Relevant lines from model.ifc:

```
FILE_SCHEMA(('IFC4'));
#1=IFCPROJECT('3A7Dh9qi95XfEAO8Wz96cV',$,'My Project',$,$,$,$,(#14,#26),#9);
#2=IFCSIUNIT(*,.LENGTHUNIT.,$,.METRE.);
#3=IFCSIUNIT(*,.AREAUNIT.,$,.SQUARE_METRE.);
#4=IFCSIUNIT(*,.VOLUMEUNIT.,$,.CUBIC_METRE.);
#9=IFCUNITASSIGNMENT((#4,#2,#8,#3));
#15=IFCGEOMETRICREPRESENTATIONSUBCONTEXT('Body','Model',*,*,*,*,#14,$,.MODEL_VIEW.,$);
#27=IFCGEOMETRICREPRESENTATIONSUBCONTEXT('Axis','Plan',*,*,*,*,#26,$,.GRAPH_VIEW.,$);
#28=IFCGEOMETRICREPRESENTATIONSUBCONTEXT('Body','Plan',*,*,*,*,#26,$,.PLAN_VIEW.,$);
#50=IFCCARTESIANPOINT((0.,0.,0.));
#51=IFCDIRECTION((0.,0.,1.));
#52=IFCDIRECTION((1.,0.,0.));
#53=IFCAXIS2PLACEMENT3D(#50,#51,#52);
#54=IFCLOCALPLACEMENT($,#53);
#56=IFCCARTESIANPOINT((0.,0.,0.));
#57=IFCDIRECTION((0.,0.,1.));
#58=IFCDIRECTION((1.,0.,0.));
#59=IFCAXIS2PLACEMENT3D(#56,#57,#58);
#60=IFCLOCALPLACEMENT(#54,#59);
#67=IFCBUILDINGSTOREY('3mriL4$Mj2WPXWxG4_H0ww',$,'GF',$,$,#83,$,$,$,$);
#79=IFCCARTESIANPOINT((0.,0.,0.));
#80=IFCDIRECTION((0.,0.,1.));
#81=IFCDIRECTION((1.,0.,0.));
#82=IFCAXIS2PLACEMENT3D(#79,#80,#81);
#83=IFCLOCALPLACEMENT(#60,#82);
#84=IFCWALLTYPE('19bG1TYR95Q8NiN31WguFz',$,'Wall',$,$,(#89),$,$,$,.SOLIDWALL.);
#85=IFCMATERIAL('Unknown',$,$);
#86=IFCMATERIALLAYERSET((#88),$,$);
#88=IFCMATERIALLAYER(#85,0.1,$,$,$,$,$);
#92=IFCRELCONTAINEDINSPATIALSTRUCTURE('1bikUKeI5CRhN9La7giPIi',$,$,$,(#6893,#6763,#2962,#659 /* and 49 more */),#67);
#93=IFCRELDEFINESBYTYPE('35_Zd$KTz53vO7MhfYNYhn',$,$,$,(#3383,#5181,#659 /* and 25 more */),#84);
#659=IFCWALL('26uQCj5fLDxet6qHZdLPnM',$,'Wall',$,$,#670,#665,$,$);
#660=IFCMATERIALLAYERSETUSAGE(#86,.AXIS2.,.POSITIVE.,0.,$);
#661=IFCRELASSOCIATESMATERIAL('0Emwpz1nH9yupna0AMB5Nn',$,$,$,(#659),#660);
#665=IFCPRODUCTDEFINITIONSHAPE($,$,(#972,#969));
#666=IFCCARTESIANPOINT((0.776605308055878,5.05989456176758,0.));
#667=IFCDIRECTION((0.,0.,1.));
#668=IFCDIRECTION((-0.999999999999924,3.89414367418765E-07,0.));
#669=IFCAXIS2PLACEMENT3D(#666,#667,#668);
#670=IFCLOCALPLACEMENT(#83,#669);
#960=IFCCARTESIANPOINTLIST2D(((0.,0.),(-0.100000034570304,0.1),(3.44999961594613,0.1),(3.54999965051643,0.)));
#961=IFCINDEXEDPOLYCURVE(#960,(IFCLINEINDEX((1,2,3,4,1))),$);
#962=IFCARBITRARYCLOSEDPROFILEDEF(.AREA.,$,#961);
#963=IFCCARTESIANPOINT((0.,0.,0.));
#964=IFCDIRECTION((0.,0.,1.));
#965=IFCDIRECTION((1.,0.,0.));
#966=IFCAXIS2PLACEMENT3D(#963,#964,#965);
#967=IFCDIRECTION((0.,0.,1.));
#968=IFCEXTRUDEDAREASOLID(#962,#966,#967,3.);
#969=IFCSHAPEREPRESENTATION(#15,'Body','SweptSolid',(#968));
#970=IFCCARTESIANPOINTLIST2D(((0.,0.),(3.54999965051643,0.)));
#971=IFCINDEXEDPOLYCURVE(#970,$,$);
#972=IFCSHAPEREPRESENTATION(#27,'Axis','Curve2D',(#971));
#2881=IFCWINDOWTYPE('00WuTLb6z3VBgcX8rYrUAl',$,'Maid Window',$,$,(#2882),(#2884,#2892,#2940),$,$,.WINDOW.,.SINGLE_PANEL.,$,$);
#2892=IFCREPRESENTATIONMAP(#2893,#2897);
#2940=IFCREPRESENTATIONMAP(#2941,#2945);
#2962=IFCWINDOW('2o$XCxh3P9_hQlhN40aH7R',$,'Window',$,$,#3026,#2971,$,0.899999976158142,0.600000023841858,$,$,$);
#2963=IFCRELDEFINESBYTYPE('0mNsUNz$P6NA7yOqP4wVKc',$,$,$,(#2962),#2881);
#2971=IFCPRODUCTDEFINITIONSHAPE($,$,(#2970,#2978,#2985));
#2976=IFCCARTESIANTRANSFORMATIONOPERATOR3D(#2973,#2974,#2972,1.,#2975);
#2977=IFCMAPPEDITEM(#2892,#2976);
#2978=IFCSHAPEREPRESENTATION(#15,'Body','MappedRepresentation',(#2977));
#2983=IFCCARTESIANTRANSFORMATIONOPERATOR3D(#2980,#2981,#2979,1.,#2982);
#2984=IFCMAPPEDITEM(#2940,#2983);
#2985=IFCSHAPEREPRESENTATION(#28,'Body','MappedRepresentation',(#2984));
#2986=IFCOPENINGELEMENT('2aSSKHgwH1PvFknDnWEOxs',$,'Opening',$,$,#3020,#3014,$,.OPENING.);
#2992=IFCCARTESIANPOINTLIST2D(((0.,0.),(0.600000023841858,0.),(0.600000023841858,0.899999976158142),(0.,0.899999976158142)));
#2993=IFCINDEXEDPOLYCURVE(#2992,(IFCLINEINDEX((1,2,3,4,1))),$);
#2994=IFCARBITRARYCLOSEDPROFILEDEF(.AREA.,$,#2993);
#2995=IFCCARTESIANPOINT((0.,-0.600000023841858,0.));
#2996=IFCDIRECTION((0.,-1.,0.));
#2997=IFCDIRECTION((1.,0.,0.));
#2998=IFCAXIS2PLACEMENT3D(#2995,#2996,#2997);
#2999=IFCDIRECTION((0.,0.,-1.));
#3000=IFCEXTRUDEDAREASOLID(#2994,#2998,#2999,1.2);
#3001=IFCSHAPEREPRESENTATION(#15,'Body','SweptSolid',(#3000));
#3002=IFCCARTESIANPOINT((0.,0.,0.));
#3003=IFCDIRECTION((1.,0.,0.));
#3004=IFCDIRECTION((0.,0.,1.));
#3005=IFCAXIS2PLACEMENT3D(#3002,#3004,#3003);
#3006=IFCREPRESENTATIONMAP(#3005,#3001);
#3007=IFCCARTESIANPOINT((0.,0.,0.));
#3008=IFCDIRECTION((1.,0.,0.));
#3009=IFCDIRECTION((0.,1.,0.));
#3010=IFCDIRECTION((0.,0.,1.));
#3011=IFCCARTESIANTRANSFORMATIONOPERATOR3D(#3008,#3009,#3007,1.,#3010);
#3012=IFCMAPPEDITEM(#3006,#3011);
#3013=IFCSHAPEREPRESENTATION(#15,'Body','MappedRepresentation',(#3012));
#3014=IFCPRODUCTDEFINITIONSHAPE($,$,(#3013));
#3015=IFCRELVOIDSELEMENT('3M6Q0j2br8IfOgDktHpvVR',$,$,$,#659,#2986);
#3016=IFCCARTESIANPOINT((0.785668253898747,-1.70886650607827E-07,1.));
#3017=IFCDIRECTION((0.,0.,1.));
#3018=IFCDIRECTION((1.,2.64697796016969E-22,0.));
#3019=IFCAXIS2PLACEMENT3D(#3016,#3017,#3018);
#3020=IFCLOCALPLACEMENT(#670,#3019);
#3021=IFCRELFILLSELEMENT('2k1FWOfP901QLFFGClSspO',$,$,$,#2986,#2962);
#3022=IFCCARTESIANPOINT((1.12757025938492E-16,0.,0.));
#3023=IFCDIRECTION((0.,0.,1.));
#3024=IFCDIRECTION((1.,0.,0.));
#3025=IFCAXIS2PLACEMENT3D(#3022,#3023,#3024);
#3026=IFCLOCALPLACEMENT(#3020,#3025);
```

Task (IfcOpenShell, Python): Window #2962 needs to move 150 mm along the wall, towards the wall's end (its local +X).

```python
import ifcopenshell
import ifcopenshell.api.geometry
import ifcopenshell.util.placement

model = ifcopenshell.open("model.ifc")

window = model.by_id(2962)
opening = window.FillsVoids[0].RelatingOpeningElement
wall = opening.VoidsElements[0].RelatingBuildingElement

wall_matrix = ifcopenshell.util.placement.get_local_placement(wall.ObjectPlacement)
shift = wall_matrix[:3, 0] * 0.15
before = ifcopenshell.util.placement.get_local_placement(window.ObjectPlacement)[:3, 3].copy()

# The window is placed relative to its opening, so it follows when the opening moves.
matrix = ifcopenshell.util.placement.get_local_placement(opening.ObjectPlacement)
matrix[:3, 3] += shift
ifcopenshell.api.geometry.edit_object_placement(
    model, product=opening, matrix=matrix, is_si=False, should_transform_children=True
)

after = ifcopenshell.util.placement.get_local_placement(window.ObjectPlacement)[:3, 3]
print("window moved by", (after - before).round(3) + 0.0)

model.write("model_edited.ifc")
```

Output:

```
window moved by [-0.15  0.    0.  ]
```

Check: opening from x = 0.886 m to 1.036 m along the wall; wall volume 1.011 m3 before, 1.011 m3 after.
